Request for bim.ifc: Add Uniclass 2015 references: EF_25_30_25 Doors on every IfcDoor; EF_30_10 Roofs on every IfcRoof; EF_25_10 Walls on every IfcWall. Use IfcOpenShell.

First a look at what the model holds.

```python
import ifcopenshell

model = ifcopenshell.open("bim.ifc")
print(model.schema)
print("classifications:", [c.Name for c in model.by_type("IfcClassification")])
for ifc_class in ("IfcDoor", "IfcRoof", "IfcStair", "IfcWall", "IfcWindow"):
    print(ifc_class, len(model.by_type(ifc_class)))
```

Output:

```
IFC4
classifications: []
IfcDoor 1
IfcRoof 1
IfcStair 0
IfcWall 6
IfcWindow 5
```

```python
import ifcopenshell
import ifcopenshell.api.classification

model = ifcopenshell.open("bim.ifc")

system = ifcopenshell.api.classification.add_classification(model, classification="Uniclass 2015")

codes = {
    "IfcDoor": ("EF_25_30_25", "Doors"),
    "IfcRoof": ("EF_30_10", "Roofs"),
    "IfcWall": ("EF_25_10", "Walls"),
}
for ifc_class, (code, name) in codes.items():
    products = model.by_type(ifc_class)
    ifcopenshell.api.classification.add_reference(
        model, products=products, classification=system, identification=code, name=name
    )
    print(code, len(products))

model.write("bim_edited.ifc")
```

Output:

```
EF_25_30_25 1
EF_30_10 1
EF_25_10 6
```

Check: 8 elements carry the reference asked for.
